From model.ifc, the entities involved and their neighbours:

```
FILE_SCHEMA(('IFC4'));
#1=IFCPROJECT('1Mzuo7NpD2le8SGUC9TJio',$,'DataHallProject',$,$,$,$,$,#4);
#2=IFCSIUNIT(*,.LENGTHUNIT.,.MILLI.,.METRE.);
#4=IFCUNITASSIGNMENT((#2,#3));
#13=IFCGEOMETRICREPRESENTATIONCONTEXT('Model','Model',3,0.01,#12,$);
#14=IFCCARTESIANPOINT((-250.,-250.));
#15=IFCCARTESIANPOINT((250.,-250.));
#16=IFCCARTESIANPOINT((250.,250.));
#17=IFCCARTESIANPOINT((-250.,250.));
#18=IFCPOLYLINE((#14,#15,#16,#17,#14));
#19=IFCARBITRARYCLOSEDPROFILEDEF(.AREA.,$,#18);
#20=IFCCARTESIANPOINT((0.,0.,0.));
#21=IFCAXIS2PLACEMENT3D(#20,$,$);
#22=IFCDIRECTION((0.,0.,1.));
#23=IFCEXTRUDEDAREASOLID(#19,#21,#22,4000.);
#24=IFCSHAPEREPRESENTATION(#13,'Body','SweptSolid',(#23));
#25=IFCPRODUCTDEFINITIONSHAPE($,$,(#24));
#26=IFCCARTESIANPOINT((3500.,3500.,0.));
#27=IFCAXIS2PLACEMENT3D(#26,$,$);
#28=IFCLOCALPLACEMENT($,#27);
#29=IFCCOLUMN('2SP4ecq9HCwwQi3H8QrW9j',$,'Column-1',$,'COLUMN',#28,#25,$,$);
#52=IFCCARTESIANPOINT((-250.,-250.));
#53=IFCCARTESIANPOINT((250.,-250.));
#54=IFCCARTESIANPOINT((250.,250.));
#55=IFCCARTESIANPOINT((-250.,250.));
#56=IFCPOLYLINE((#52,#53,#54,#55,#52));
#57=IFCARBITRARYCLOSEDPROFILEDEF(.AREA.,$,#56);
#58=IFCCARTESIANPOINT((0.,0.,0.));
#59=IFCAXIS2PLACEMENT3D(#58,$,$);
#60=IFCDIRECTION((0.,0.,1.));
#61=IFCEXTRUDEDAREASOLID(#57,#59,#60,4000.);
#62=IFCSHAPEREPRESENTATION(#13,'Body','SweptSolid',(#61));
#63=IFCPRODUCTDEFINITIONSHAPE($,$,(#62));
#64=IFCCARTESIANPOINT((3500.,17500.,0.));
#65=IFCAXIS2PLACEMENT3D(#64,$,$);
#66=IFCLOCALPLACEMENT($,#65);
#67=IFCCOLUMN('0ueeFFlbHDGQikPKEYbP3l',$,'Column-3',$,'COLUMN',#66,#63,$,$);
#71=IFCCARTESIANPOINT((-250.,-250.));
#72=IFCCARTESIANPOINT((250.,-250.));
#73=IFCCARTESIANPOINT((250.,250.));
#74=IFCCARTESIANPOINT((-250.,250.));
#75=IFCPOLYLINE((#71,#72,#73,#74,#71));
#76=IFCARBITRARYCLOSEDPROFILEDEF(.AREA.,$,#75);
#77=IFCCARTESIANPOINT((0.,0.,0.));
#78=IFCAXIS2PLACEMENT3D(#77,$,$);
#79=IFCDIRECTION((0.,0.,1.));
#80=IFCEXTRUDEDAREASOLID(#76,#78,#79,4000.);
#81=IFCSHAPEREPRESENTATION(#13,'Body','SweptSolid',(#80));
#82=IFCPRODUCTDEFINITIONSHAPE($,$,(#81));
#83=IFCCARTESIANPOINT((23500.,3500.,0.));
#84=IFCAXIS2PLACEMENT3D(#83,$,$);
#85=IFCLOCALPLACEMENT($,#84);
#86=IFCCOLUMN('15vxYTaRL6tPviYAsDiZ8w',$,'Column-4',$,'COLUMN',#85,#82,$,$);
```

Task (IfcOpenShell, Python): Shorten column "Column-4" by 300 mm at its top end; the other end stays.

```python
import ifcopenshell

model = ifcopenshell.open("model.ifc")

member = model.by_id(86)
change = -300.0

# The extrusion runs towards the end named, so only its depth changes.
body = next(r for r in member.Representation.Representations if r.RepresentationIdentifier == "Body")
solid = body.Items[0]
old_length = solid.Depth
solid.Depth += change

print(f"length {old_length:g} -> {solid.Depth:g}")

model.write("model_v2.ifc")
```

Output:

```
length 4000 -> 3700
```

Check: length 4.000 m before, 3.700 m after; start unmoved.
